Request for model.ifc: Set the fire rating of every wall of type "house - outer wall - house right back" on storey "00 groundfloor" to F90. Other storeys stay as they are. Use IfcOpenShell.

First a look at what the model holds.

```python
import ifcopenshell
import ifcopenshell.util.element

model = ifcopenshell.open("model.ifc")
print(model.schema)
storey = next(s for s in model.by_type("IfcBuildingStorey") if s.Name == "00 groundfloor")
walls = [e for e in ifcopenshell.util.element.get_decomposition(storey) if e.is_a("IfcWall")]
seen = {}
for e in walls:
    element_type = ifcopenshell.util.element.get_type(e)
    key = (element_type.Name if element_type != e and element_type else None, ifcopenshell.util.element.get_pset(e, "Pset_WallCommon", "FireRating"))
    seen[key] = seen.get(key, 0) + 1
for (name, value), count in sorted(seen.items(), key=str):
    print(count, "x", name, "|", value)
```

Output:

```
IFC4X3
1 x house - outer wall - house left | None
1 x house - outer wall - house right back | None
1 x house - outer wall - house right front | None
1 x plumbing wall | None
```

```python
import ifcopenshell
import ifcopenshell.api.pset
import ifcopenshell.util.element

model = ifcopenshell.open("model.ifc")

storey = next(s for s in model.by_type("IfcBuildingStorey") if s.Name == "00 groundfloor")
walls = [e for e in ifcopenshell.util.element.get_decomposition(storey) if e.is_a("IfcWall")]

count = 0
for e in walls:
    element_type = ifcopenshell.util.element.get_type(e)
    if element_type in (None, e) or element_type.Name != "house - outer wall - house right back":
        continue
    # add_pset returns the element's existing set when there is one.
    pset = ifcopenshell.api.pset.add_pset(model, product=e, name="Pset_WallCommon")
    ifcopenshell.api.pset.edit_pset(model, pset=pset, properties={"FireRating": "F90"})
    count += 1

print(count, "walls updated")

model.write("model-out.ifc")
```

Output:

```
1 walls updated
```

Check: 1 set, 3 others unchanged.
